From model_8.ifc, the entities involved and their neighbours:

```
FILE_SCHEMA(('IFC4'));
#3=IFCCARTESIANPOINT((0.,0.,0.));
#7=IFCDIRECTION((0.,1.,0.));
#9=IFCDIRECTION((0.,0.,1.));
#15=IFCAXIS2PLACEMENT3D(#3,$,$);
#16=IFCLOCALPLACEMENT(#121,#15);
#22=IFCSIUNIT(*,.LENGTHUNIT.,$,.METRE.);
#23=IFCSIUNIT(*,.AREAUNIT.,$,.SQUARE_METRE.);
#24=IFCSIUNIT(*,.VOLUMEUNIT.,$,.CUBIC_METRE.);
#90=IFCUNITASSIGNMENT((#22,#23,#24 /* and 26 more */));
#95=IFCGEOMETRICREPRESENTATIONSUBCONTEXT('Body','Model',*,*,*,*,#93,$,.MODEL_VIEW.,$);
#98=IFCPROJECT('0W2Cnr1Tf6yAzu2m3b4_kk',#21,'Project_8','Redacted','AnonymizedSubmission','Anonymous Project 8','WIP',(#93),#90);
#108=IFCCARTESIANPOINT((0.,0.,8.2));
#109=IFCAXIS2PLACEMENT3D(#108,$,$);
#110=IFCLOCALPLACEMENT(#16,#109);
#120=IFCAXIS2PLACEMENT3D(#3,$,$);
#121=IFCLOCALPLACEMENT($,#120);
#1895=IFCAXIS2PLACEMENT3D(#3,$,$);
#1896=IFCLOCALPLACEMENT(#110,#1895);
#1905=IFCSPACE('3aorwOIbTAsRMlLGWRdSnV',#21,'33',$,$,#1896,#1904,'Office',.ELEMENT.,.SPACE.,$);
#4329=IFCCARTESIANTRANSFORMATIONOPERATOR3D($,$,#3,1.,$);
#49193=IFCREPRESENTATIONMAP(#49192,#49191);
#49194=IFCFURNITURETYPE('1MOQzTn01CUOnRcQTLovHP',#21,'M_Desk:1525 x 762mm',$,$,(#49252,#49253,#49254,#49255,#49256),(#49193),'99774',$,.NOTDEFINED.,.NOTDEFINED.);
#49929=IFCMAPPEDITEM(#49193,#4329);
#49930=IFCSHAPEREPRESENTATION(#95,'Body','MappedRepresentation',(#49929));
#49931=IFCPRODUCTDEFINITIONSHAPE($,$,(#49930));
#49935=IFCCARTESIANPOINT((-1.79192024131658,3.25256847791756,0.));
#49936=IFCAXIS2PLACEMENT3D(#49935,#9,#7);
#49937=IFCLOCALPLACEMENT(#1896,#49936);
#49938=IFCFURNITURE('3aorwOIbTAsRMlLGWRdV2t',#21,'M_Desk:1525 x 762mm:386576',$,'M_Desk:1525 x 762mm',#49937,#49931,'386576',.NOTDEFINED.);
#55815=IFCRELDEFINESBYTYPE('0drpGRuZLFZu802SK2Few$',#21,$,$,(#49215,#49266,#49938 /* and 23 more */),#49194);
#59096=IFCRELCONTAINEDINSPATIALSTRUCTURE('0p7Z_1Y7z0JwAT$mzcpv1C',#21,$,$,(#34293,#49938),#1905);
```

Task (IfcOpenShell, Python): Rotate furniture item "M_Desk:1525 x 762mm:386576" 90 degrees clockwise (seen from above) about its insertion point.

```python
import ifcopenshell
import ifcopenshell.api.geometry
import ifcopenshell.util.placement

model = ifcopenshell.open("model_8.ifc")

item = model.by_guid("3aorwOIbTAsRMlLGWRdV2t")
matrix = ifcopenshell.util.placement.get_local_placement(item.ObjectPlacement)
matrix = matrix @ ifcopenshell.util.placement.rotation(-90, "Z")
ifcopenshell.api.geometry.edit_object_placement(model, product=item, matrix=matrix, is_si=False)

print(ifcopenshell.util.placement.get_local_placement(item.ObjectPlacement).round(3) + 0.0)

model.write("model_8_rev.ifc")
```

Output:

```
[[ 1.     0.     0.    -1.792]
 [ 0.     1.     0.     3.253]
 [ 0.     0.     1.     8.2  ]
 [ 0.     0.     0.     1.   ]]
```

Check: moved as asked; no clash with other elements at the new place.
